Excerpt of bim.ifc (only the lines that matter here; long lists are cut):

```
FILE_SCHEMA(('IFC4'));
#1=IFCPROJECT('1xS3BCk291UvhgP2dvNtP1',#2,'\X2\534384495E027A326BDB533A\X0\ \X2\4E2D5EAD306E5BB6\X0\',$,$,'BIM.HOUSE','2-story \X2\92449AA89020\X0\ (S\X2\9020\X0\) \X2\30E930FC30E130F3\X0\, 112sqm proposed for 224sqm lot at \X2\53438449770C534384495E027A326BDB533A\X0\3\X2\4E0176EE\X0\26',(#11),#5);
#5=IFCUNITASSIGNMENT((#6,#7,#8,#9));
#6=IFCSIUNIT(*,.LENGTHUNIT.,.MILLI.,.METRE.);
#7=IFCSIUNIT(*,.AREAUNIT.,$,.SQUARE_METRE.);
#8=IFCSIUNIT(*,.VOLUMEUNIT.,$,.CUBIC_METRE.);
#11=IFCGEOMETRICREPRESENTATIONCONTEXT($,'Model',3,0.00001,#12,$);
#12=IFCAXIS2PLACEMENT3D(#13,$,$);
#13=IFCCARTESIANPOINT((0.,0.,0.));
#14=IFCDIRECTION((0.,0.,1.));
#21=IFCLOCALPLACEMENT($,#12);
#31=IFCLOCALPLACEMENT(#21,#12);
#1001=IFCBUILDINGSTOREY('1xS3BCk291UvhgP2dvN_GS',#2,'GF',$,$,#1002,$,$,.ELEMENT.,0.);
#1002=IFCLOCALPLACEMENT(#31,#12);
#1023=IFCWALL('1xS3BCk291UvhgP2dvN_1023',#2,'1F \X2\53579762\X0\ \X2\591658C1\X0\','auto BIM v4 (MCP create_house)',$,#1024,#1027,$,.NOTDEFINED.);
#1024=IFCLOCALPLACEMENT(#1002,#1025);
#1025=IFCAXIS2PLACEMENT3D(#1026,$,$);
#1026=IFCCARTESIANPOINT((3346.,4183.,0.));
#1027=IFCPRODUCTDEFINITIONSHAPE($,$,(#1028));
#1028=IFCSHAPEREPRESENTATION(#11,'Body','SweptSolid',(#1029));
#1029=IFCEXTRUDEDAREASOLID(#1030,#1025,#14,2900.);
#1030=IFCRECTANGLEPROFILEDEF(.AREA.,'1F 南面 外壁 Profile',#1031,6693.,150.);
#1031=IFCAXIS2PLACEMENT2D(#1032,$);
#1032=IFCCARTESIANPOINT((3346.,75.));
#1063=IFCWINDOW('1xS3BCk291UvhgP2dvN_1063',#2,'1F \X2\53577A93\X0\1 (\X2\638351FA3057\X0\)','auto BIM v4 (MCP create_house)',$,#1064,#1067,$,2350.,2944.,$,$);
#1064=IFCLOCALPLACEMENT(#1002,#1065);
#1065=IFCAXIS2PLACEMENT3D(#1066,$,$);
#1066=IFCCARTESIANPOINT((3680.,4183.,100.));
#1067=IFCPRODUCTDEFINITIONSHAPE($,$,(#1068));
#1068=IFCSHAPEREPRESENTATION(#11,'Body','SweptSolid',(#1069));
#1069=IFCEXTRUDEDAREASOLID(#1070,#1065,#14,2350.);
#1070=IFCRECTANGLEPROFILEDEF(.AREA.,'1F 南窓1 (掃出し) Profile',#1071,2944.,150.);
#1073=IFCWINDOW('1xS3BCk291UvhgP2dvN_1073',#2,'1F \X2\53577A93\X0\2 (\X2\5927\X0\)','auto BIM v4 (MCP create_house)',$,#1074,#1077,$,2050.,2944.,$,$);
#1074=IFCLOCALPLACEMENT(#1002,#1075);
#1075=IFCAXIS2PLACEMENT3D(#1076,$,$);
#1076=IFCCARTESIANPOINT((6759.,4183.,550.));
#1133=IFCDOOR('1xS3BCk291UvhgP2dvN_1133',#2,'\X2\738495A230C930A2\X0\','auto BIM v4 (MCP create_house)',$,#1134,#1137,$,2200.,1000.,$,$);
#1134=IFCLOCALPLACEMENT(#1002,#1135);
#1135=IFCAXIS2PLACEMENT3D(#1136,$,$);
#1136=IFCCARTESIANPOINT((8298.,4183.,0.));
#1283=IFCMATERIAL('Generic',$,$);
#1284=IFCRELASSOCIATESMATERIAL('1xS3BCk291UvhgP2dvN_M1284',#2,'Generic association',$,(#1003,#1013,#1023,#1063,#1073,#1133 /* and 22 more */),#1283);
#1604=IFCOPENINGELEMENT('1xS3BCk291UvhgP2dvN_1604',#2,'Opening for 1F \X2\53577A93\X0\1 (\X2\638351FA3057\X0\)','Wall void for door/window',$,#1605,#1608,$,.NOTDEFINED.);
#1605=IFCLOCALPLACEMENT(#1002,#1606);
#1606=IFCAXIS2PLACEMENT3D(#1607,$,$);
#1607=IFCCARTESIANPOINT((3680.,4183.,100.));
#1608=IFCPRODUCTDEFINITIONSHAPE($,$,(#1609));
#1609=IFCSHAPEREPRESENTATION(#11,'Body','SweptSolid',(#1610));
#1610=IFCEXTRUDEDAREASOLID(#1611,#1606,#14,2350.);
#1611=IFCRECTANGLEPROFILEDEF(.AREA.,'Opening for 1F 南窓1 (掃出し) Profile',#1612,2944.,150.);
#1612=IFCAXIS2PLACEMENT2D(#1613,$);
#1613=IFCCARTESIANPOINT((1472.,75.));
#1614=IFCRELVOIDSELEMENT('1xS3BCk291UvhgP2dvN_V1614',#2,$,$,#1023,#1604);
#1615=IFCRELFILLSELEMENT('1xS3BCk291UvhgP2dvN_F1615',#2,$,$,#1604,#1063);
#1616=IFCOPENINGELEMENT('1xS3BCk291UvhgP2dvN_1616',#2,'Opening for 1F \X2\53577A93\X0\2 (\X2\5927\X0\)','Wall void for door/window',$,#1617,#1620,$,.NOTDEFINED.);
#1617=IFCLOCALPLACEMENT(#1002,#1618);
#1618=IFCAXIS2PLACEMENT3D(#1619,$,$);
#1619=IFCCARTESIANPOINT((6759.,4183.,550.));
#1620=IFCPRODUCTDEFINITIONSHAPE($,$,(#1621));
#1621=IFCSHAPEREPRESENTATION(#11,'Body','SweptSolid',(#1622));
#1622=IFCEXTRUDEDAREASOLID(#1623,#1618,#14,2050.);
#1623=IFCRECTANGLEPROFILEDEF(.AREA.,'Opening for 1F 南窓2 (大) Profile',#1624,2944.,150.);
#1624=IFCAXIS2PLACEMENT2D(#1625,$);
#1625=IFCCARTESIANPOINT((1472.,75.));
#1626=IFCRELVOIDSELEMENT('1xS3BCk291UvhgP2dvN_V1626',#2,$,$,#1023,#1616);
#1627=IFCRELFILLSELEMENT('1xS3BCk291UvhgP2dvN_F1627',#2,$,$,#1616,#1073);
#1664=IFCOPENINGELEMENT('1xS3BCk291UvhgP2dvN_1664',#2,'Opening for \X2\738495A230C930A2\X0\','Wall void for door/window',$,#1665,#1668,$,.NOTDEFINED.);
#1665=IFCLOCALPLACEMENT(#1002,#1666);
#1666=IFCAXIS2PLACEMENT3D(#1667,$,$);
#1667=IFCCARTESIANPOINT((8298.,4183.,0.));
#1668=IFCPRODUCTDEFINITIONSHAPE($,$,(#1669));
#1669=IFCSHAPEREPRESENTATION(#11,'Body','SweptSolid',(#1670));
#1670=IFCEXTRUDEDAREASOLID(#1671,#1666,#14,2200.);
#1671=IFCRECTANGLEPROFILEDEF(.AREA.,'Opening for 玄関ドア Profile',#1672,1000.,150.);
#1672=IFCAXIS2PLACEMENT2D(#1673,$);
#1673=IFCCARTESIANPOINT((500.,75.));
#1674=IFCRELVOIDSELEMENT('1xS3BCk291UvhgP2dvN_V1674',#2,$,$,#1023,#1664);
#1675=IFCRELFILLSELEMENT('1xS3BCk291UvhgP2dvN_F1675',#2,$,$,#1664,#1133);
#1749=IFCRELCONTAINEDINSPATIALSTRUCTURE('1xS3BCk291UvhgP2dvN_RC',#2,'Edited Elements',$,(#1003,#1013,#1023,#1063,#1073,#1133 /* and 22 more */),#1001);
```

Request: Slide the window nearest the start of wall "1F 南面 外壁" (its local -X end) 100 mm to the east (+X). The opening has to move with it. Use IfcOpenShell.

```python
import ifcopenshell
import ifcopenshell.api.geometry
import ifcopenshell.util.placement

model = ifcopenshell.open("bim.ifc")

window = model.by_id(1063)
opening = window.FillsVoids[0].RelatingOpeningElement
wall = opening.VoidsElements[0].RelatingBuildingElement

wall_matrix = ifcopenshell.util.placement.get_local_placement(wall.ObjectPlacement)
shift = wall_matrix[:3, 0] * 100.0
before = ifcopenshell.util.placement.get_local_placement(window.ObjectPlacement)[:3, 3].copy()

# The window is not placed relative to its opening, so move both.
for product in (opening, window):
    matrix = ifcopenshell.util.placement.get_local_placement(product.ObjectPlacement)
    matrix[:3, 3] += shift
    ifcopenshell.api.geometry.edit_object_placement(model, product=product, matrix=matrix, is_si=False)

after = ifcopenshell.util.placement.get_local_placement(window.ObjectPlacement)[:3, 3]
print("window moved by", (after - before).round(3) + 0.0)

model.write("bim_rev.ifc")
```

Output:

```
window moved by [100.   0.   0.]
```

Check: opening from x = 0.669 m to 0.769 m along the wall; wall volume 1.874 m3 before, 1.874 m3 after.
